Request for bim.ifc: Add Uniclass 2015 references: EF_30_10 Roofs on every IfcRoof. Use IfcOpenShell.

First a look at what the model holds.

```python
import ifcopenshell

model = ifcopenshell.open("bim.ifc")
print(model.schema)
print("classifications:", [c.Name for c in model.by_type("IfcClassification")])
for ifc_class in ("IfcDoor", "IfcRoof", "IfcStair", "IfcWall", "IfcWindow"):
    print(ifc_class, len(model.by_type(ifc_class)))
```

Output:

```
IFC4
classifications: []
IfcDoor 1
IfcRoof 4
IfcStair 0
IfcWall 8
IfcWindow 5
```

```python
import ifcopenshell
import ifcopenshell.api.classification

model = ifcopenshell.open("bim.ifc")

system = ifcopenshell.api.classification.add_classification(model, classification="Uniclass 2015")

codes = {
    "IfcRoof": ("EF_30_10", "Roofs"),
}
for ifc_class, (code, name) in codes.items():
    products = model.by_type(ifc_class)
    ifcopenshell.api.classification.add_reference(
        model, products=products, classification=system, identification=code, name=name
    )
    print(code, len(products))

model.write("bim_edited.ifc")
```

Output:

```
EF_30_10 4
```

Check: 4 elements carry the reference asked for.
